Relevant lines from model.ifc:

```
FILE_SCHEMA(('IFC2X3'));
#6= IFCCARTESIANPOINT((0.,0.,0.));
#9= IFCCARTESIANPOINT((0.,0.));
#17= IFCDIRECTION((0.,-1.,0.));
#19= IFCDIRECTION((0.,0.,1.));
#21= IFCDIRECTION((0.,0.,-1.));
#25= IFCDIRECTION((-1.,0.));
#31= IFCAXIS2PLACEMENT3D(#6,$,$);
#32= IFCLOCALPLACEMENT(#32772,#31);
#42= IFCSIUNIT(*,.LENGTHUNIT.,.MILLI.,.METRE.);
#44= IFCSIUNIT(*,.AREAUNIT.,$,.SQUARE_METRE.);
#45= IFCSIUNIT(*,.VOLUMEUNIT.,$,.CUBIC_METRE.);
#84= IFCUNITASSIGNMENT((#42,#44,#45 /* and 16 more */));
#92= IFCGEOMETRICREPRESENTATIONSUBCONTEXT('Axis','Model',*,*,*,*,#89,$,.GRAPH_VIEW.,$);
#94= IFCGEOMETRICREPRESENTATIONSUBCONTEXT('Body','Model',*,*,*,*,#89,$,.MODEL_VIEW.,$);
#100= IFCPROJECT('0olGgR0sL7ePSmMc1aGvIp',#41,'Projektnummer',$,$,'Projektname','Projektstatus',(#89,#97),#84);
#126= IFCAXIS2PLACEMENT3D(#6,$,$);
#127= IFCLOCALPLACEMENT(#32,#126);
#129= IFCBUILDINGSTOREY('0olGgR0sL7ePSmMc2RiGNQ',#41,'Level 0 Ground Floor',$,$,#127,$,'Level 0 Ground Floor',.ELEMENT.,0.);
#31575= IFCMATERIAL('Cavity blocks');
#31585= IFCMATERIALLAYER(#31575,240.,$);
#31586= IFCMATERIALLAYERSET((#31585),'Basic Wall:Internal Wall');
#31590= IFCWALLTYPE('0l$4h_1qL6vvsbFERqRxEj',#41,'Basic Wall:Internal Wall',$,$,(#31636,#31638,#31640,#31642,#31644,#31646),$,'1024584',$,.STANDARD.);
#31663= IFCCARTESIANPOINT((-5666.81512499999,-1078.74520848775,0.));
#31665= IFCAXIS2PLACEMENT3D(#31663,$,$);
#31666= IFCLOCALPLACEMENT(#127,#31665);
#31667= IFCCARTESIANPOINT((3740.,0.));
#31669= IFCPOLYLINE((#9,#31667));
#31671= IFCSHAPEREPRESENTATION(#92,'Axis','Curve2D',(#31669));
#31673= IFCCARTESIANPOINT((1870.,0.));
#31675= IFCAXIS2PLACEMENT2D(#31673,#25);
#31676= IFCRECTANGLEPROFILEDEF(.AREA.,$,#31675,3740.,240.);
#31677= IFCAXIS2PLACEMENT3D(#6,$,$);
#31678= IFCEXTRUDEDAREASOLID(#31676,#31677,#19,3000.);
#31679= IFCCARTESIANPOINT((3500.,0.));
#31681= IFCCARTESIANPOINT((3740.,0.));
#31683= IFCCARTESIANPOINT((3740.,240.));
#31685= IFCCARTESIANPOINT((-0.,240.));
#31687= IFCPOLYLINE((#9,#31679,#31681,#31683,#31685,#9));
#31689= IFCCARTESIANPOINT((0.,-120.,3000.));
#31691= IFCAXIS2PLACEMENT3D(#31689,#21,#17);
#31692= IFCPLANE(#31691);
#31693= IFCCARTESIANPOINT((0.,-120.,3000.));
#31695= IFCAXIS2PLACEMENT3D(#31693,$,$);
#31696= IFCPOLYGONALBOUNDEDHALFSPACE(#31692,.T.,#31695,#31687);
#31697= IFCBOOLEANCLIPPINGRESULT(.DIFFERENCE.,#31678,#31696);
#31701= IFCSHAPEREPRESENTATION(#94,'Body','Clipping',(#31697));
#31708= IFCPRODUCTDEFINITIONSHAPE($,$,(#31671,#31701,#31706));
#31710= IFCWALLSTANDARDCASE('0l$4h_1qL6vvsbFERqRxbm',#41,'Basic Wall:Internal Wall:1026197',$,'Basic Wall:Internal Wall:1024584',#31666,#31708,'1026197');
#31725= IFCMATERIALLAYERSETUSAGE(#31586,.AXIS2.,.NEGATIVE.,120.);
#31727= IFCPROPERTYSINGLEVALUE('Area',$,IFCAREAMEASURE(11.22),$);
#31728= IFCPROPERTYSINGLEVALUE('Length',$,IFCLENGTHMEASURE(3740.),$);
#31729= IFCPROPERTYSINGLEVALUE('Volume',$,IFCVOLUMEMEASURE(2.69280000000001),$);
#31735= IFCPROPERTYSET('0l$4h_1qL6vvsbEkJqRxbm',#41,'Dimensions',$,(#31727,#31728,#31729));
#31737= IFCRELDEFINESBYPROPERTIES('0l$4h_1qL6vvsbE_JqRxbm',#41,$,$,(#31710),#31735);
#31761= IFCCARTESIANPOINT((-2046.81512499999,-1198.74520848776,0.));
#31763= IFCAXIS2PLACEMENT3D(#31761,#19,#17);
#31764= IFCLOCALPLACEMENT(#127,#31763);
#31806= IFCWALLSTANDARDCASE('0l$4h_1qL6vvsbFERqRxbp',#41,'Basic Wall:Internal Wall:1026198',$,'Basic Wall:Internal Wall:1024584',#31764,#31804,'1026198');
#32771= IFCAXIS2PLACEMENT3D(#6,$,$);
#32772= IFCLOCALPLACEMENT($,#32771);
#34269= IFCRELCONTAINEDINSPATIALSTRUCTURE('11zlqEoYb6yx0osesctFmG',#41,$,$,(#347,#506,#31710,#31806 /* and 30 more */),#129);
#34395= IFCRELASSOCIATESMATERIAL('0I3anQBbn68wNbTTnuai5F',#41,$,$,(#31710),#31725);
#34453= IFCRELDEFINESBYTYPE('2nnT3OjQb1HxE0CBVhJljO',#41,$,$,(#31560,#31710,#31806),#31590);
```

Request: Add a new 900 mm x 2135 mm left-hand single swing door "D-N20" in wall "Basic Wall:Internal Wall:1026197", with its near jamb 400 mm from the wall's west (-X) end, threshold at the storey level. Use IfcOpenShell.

```python
import numpy as np
import ifcopenshell
import ifcopenshell.api.feature
import ifcopenshell.api.geometry
import ifcopenshell.api.pset
import ifcopenshell.api.root
import ifcopenshell.api.spatial
import ifcopenshell.api.type
import ifcopenshell.geom
import ifcopenshell.util.element
import ifcopenshell.util.placement
import ifcopenshell.util.representation
import ifcopenshell.util.shape
import ifcopenshell.util.unit

model = ifcopenshell.open("model.ifc")
unit_scale = ifcopenshell.util.unit.calculate_unit_scale(model)
area_scale = ifcopenshell.util.unit.calculate_unit_scale(model, "AREAUNIT")
volume_scale = ifcopenshell.util.unit.calculate_unit_scale(model, "VOLUMEUNIT")
settings = ifcopenshell.geom.settings()


def volume(element):
    """Net volume in cubic metres, openings subtracted."""
    shape = ifcopenshell.geom.create_shape(settings, element)
    return ifcopenshell.util.shape.get_volume(shape.geometry)


wall = model.by_guid("0l$4h_1qL6vvsbFERqRxbm")
storey = ifcopenshell.util.element.get_container(wall, ifc_class="IfcBuildingStorey")
context = ifcopenshell.util.representation.get_context(model, "Model", "Body", "MODEL_VIEW")
before = volume(wall)

width, height, from_end, sill = 0.9, 2.135, 0.4, 0.0  # metres

# The wall runs along its own X axis, and the end named is its -X end.
wall_shape = ifcopenshell.geom.create_shape(settings, wall)
x, y, z = ifcopenshell.util.shape.get_vertices(wall_shape.geometry).T
start = x.min() + from_end
face, thickness = float(y.min()), float(y.max() - y.min())
wall_matrix = ifcopenshell.util.placement.get_local_placement(wall.ObjectPlacement)
level = ifcopenshell.util.placement.get_local_placement(storey.ObjectPlacement)[2, 3]


def in_wall(x, y):
    """Placement at x, y metres in the wall's axes, at sill height."""
    matrix = wall_matrix.copy()
    matrix[:, 3] = wall_matrix @ np.array([x / unit_scale, y / unit_scale, 0.0, 1.0])
    matrix[2, 3] = level + sill / unit_scale
    return matrix


# Opening: a box that overshoots both wall faces by 50 mm.
opening = ifcopenshell.api.root.create_entity(model, ifc_class="IfcOpeningElement")
box = ifcopenshell.api.geometry.add_wall_representation(
    model, context=context, length=width, height=height, thickness=thickness + 0.1
)
ifcopenshell.api.geometry.assign_representation(model, product=opening, representation=box)
ifcopenshell.api.geometry.edit_object_placement(model, product=opening, matrix=in_wall(start, face - 0.05), is_si=False)
ifcopenshell.api.feature.add_feature(model, feature=opening, element=wall)

door = ifcopenshell.api.root.create_entity(model, ifc_class="IfcDoor", name="D-N20")
door.OverallWidth, door.OverallHeight = width / unit_scale, height / unit_scale
body = ifcopenshell.api.geometry.add_door_representation(
    model,
    context=context,
    overall_width=door.OverallWidth,
    overall_height=door.OverallHeight,
    operation_type="SINGLE_SWING_LEFT",
    lining_properties={"LiningDepth": thickness / unit_scale, "ThresholdDepth": thickness / unit_scale},
)
ifcopenshell.api.geometry.assign_representation(model, product=door, representation=body)
ifcopenshell.api.spatial.assign_container(model, products=[door], relating_structure=storey)
fills = ifcopenshell.api.feature.add_filling(model, opening=opening, element=door)
fills.OwnerHistory = door.OwnerHistory  # required in IFC2X3

# IFC2X3 keeps the operation on the door style.
style = ifcopenshell.api.root.create_entity(model, ifc_class="IfcDoorStyle", name="D-N20")
style.OperationType, style.ConstructionType = "SINGLE_SWING_LEFT", "NOTDEFINED"
style.ParameterTakesPrecedence = style.Sizeable = False
ifcopenshell.api.type.assign_type(model, related_objects=[door], relating_type=style)

# The lining spans the wall, so the door starts at the wall face.
ifcopenshell.api.geometry.edit_object_placement(model, product=door, matrix=in_wall(start, face), is_si=False)

after = volume(wall)

# Update the wall's stored quantities.
pset = model.by_id(ifcopenshell.util.element.get_pset(wall, "Dimensions", should_inherit=False)["id"])
ifcopenshell.api.pset.edit_pset(model, pset=pset, properties={
    "Area": model.create_entity("IfcAreaMeasure", after / thickness / area_scale),
    "Volume": model.create_entity("IfcVolumeMeasure", after / volume_scale),
})

print(f"wall volume {before:.3f} -> {after:.3f} m3")

model.write("model_rev.ifc")
```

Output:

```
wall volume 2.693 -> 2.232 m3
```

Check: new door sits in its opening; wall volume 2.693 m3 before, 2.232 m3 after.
